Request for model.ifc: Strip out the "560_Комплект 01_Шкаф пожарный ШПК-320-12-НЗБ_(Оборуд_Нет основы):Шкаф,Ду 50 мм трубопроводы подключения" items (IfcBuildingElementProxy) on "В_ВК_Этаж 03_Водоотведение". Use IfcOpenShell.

First a look at what the model holds.

```python
import ifcopenshell
import ifcopenshell.util.element

model = ifcopenshell.open("model.ifc")
print(model.schema)
storey = next(s for s in model.by_type("IfcBuildingStorey") if s.Name == "В_ВК_Этаж 03_Водоотведение")
proxies = [e for e in ifcopenshell.util.element.get_decomposition(storey) if e.is_a("IfcBuildingElementProxy")]
seen = {}
for e in proxies:
    element_type = ifcopenshell.util.element.get_type(e)
    name = element_type.Name if element_type not in (None, e) else None
    seen[name] = seen.get(name, 0) + 1
for name, count in sorted(seen.items(), key=str):
    print(count, "x", name)
```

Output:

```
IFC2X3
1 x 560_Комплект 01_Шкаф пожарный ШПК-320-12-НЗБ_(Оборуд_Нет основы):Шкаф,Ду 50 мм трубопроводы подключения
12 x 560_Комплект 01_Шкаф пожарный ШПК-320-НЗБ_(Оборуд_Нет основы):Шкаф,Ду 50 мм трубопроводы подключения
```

```python
import ifcopenshell
import ifcopenshell.api.root
import ifcopenshell.util.element

model = ifcopenshell.open("model.ifc")

storey = next(s for s in model.by_type("IfcBuildingStorey") if s.Name == "В_ВК_Этаж 03_Водоотведение")
proxies = [e for e in ifcopenshell.util.element.get_decomposition(storey) if e.is_a("IfcBuildingElementProxy")]
targets = [e for e in proxies if (t := ifcopenshell.util.element.get_type(e)) not in (None, e) and t.Name == "560_Комплект 01_Шкаф пожарный ШПК-320-12-НЗБ_(Оборуд_Нет основы):Шкаф,Ду 50 мм трубопроводы подключения"]

for e in targets:
    ifcopenshell.api.root.remove_product(model, product=e)
print(len(targets), "removed")

model.write("model_rev.ifc")
```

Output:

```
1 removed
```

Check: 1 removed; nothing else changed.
